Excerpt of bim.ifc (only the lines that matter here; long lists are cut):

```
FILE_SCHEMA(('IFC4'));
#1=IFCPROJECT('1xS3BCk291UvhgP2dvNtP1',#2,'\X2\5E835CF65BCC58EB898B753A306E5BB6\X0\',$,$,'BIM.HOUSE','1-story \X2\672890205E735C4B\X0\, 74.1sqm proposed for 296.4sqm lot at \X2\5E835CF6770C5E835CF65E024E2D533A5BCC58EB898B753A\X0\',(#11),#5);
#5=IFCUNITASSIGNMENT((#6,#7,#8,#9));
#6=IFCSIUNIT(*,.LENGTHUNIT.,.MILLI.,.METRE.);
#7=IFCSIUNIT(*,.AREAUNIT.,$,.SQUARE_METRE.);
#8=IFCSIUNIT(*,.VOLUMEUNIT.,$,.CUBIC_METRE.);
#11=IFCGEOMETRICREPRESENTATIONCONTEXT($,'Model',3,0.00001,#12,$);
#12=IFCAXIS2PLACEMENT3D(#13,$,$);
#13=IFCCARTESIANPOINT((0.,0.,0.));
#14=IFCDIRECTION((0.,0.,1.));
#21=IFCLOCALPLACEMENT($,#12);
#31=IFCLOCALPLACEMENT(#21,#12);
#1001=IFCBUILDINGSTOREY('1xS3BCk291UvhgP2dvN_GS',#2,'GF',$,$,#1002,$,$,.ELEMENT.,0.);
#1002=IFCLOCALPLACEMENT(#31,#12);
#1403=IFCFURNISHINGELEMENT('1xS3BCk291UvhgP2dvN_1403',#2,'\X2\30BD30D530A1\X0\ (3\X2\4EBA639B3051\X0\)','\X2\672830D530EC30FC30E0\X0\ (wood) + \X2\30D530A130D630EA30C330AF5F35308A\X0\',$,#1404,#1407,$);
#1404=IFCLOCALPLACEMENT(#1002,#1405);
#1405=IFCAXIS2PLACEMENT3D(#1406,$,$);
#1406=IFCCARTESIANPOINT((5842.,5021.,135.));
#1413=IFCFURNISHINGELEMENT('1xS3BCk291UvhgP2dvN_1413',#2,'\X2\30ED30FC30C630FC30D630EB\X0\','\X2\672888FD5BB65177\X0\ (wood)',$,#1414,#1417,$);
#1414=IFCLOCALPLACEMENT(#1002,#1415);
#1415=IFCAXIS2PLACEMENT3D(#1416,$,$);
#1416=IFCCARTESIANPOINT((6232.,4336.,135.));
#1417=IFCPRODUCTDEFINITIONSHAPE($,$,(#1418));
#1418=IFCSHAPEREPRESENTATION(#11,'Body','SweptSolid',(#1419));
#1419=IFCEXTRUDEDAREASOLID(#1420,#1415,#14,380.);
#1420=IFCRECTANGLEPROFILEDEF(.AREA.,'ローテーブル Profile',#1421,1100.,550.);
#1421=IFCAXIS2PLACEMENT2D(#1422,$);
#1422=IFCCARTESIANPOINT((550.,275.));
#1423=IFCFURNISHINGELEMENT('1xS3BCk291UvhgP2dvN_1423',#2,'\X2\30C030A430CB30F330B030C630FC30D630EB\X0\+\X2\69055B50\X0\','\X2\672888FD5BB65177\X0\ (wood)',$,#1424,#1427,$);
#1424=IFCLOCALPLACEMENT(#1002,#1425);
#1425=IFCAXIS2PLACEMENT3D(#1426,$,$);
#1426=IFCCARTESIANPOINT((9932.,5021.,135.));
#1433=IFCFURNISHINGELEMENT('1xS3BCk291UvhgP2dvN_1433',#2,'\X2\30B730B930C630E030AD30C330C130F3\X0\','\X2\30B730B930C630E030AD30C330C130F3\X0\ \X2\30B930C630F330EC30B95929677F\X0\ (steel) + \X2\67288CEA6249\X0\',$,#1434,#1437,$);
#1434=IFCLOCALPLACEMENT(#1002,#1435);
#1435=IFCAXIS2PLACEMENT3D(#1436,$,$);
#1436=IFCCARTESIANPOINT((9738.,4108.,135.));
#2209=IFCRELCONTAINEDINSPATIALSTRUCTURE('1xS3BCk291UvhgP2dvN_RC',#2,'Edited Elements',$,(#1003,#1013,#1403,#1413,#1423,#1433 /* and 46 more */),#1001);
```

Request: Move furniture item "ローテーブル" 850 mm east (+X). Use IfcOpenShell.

```python
import ifcopenshell
import ifcopenshell.api.geometry
import ifcopenshell.util.placement
import ifcopenshell.util.unit

model = ifcopenshell.open("bim.ifc")
unit_scale = ifcopenshell.util.unit.calculate_unit_scale(model)

item = model.by_guid("1xS3BCk291UvhgP2dvN_1413")
matrix = ifcopenshell.util.placement.get_local_placement(item.ObjectPlacement)
matrix[0, 3] += 0.85 / unit_scale
ifcopenshell.api.geometry.edit_object_placement(model, product=item, matrix=matrix, is_si=False)

print(ifcopenshell.util.placement.get_local_placement(item.ObjectPlacement).round(3) + 0.0)

model.write("bim-out.ifc")
```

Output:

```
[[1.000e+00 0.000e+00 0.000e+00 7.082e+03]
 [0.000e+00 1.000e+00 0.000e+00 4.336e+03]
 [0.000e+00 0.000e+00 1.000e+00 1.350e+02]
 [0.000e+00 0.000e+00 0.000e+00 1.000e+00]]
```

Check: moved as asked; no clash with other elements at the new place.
